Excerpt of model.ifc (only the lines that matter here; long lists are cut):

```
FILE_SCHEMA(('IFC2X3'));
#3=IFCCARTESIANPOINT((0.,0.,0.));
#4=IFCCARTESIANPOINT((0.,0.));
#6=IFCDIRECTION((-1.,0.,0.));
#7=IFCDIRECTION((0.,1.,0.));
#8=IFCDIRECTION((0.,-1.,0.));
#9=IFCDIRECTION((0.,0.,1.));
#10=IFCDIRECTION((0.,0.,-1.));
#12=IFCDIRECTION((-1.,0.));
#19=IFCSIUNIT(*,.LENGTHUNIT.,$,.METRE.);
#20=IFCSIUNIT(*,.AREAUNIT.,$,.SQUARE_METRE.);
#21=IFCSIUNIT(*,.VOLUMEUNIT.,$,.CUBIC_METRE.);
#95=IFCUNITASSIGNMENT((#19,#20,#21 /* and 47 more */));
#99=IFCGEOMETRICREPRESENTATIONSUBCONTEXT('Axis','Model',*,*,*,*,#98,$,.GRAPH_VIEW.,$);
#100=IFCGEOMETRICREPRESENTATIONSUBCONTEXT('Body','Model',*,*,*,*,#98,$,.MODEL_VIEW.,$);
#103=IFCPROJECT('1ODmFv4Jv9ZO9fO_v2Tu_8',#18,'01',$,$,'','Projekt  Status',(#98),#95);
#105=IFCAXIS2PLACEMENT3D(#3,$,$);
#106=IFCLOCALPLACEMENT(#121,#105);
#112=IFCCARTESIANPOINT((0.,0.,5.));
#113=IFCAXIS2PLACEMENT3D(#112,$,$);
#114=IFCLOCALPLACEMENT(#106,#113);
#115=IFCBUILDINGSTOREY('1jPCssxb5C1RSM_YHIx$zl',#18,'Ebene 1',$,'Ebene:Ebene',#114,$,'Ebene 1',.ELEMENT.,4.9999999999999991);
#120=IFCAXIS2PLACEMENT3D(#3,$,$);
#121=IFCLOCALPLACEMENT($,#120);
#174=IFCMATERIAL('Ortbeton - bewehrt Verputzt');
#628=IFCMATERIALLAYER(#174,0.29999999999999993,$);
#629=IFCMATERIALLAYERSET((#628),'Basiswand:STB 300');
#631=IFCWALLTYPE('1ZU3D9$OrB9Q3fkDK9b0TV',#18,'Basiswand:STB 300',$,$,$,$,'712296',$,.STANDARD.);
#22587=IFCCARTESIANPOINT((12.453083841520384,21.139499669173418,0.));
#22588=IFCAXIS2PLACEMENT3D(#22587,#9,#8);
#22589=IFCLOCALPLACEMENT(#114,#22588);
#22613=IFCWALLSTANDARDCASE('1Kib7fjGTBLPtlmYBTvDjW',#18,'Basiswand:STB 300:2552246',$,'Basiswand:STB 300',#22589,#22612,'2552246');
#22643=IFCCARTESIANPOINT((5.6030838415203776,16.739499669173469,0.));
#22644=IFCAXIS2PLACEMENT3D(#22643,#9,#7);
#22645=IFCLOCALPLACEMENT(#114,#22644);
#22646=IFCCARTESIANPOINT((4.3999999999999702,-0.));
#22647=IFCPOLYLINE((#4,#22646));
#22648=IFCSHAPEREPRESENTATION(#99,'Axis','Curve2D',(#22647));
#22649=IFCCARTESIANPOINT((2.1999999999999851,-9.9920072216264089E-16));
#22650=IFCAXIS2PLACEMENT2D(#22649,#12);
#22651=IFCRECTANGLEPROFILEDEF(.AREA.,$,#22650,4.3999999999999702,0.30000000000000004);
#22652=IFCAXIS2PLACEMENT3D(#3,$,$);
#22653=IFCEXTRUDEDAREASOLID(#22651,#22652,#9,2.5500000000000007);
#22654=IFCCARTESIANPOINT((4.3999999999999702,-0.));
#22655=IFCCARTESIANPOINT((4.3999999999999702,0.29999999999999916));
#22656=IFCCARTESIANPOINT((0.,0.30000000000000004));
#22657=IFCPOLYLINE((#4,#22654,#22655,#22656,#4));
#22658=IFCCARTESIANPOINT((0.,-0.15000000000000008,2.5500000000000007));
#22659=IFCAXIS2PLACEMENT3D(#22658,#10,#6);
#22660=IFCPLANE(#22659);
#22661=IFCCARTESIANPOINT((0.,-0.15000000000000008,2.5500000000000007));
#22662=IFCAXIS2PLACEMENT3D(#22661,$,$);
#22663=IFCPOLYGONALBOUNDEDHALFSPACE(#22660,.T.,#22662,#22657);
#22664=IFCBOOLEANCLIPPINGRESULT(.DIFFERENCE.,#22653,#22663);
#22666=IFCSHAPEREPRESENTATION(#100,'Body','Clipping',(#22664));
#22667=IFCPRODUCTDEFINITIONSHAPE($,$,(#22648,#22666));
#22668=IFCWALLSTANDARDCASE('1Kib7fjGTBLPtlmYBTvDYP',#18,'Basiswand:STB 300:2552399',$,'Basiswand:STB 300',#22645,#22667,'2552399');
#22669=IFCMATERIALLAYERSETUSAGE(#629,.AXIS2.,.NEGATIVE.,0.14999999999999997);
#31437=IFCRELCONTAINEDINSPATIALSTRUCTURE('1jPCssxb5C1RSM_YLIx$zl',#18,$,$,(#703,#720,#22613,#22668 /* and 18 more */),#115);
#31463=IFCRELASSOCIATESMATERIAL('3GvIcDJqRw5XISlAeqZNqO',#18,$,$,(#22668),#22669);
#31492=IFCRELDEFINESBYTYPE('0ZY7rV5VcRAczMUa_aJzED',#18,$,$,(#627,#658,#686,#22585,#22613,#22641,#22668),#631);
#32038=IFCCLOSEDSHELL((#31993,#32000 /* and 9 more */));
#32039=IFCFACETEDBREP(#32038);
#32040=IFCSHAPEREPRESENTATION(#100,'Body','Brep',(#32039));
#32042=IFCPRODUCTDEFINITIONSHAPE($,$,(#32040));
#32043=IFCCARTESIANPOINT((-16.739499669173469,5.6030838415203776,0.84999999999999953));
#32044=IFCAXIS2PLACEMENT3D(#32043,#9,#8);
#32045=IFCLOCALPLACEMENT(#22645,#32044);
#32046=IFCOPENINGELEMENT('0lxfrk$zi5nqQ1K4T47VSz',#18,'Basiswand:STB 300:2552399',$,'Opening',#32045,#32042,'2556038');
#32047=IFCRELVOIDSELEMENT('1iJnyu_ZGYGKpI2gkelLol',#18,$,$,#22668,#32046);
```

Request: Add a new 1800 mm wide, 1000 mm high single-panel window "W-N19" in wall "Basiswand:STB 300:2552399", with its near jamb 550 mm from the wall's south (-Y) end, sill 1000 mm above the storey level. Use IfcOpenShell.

```python
import numpy as np
import ifcopenshell
import ifcopenshell.api.feature
import ifcopenshell.api.geometry
import ifcopenshell.api.root
import ifcopenshell.api.spatial
import ifcopenshell.api.type
import ifcopenshell.geom
import ifcopenshell.util.element
import ifcopenshell.util.placement
import ifcopenshell.util.representation
import ifcopenshell.util.shape
import ifcopenshell.util.unit

model = ifcopenshell.open("model.ifc")
unit_scale = ifcopenshell.util.unit.calculate_unit_scale(model)
settings = ifcopenshell.geom.settings()


def volume(element):
    """Net volume in cubic metres, openings subtracted."""
    shape = ifcopenshell.geom.create_shape(settings, element)
    return ifcopenshell.util.shape.get_volume(shape.geometry)


wall = model.by_guid("1Kib7fjGTBLPtlmYBTvDYP")
storey = ifcopenshell.util.element.get_container(wall, ifc_class="IfcBuildingStorey")
context = ifcopenshell.util.representation.get_context(model, "Model", "Body", "MODEL_VIEW")
before = volume(wall)

width, height, from_end, sill = 1.8, 1, 0.55, 1  # metres

# The wall runs along its own X axis, and the end named is its -X end.
wall_shape = ifcopenshell.geom.create_shape(settings, wall)
x, y, z = ifcopenshell.util.shape.get_vertices(wall_shape.geometry).T
start = x.min() + from_end
face, thickness = float(y.min()), float(y.max() - y.min())
wall_matrix = ifcopenshell.util.placement.get_local_placement(wall.ObjectPlacement)
level = ifcopenshell.util.placement.get_local_placement(storey.ObjectPlacement)[2, 3]


def in_wall(x, y):
    """Placement at x, y metres in the wall's axes, at sill height."""
    matrix = wall_matrix.copy()
    matrix[:, 3] = wall_matrix @ np.array([x / unit_scale, y / unit_scale, 0.0, 1.0])
    matrix[2, 3] = level + sill / unit_scale
    return matrix


# Opening: a box that overshoots both wall faces by 50 mm.
opening = ifcopenshell.api.root.create_entity(model, ifc_class="IfcOpeningElement")
box = ifcopenshell.api.geometry.add_wall_representation(
    model, context=context, length=width, height=height, thickness=thickness + 0.1
)
ifcopenshell.api.geometry.assign_representation(model, product=opening, representation=box)
ifcopenshell.api.geometry.edit_object_placement(model, product=opening, matrix=in_wall(start, face - 0.05), is_si=False)
ifcopenshell.api.feature.add_feature(model, feature=opening, element=wall)

window = ifcopenshell.api.root.create_entity(model, ifc_class="IfcWindow", name="W-N19")
window.OverallWidth, window.OverallHeight = width / unit_scale, height / unit_scale
body = ifcopenshell.api.geometry.add_window_representation(
    model,
    context=context,
    overall_width=window.OverallWidth,
    overall_height=window.OverallHeight,
    partition_type="SINGLE_PANEL",
)
ifcopenshell.api.geometry.assign_representation(model, product=window, representation=body)
ifcopenshell.api.spatial.assign_container(model, products=[window], relating_structure=storey)
fills = ifcopenshell.api.feature.add_filling(model, opening=opening, element=window)
fills.OwnerHistory = window.OwnerHistory  # required in IFC2X3

# IFC2X3 keeps the operation on the window style.
style = ifcopenshell.api.root.create_entity(model, ifc_class="IfcWindowStyle", name="W-N19")
style.OperationType, style.ConstructionType = "SINGLE_PANEL", "NOTDEFINED"
style.ParameterTakesPrecedence = style.Sizeable = False
ifcopenshell.api.type.assign_type(model, related_objects=[window], relating_type=style)

# Centre the window in the wall's thickness.
ifcopenshell.api.geometry.edit_object_placement(model, product=window, matrix=in_wall(start, face), is_si=False)
window_shape = ifcopenshell.geom.create_shape(settings, window)
depth = ifcopenshell.util.shape.get_vertices(window_shape.geometry)[:, 1]
offset = face + thickness / 2 - (depth.min() + depth.max()) / 2
ifcopenshell.api.geometry.edit_object_placement(model, product=window, matrix=in_wall(start, offset), is_si=False)

after = volume(wall)

print(f"wall volume {before:.3f} -> {after:.3f} m3")

model.write("model_v2.ifc")
```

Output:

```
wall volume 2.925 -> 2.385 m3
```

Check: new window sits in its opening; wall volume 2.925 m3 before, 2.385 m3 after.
